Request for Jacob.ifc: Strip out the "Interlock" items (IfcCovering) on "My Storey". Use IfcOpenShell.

First a look at what the model holds.

```python
import ifcopenshell
import ifcopenshell.util.element

model = ifcopenshell.open("Jacob.ifc")
print(model.schema)
storey = next(s for s in model.by_type("IfcBuildingStorey") if s.Name == "My Storey")
coverings = [e for e in ifcopenshell.util.element.get_decomposition(storey) if e.is_a("IfcCovering")]
seen = {}
for e in coverings:
    element_type = ifcopenshell.util.element.get_type(e)
    name = element_type.Name if element_type not in (None, e) else None
    seen[name] = seen.get(name, 0) + 1
for name, count in sorted(seen.items(), key=str):
    print(count, "x", name)
```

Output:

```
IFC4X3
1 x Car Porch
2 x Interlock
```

```python
import ifcopenshell
import ifcopenshell.api.root
import ifcopenshell.util.element

model = ifcopenshell.open("Jacob.ifc")

storey = next(s for s in model.by_type("IfcBuildingStorey") if s.Name == "My Storey")
coverings = [e for e in ifcopenshell.util.element.get_decomposition(storey) if e.is_a("IfcCovering")]
targets = [e for e in coverings if (t := ifcopenshell.util.element.get_type(e)) not in (None, e) and t.Name == "Interlock"]

for e in targets:
    ifcopenshell.api.root.remove_product(model, product=e)
print(len(targets), "removed")

model.write("Jacob_updated.ifc")
```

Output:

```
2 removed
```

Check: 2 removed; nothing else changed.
